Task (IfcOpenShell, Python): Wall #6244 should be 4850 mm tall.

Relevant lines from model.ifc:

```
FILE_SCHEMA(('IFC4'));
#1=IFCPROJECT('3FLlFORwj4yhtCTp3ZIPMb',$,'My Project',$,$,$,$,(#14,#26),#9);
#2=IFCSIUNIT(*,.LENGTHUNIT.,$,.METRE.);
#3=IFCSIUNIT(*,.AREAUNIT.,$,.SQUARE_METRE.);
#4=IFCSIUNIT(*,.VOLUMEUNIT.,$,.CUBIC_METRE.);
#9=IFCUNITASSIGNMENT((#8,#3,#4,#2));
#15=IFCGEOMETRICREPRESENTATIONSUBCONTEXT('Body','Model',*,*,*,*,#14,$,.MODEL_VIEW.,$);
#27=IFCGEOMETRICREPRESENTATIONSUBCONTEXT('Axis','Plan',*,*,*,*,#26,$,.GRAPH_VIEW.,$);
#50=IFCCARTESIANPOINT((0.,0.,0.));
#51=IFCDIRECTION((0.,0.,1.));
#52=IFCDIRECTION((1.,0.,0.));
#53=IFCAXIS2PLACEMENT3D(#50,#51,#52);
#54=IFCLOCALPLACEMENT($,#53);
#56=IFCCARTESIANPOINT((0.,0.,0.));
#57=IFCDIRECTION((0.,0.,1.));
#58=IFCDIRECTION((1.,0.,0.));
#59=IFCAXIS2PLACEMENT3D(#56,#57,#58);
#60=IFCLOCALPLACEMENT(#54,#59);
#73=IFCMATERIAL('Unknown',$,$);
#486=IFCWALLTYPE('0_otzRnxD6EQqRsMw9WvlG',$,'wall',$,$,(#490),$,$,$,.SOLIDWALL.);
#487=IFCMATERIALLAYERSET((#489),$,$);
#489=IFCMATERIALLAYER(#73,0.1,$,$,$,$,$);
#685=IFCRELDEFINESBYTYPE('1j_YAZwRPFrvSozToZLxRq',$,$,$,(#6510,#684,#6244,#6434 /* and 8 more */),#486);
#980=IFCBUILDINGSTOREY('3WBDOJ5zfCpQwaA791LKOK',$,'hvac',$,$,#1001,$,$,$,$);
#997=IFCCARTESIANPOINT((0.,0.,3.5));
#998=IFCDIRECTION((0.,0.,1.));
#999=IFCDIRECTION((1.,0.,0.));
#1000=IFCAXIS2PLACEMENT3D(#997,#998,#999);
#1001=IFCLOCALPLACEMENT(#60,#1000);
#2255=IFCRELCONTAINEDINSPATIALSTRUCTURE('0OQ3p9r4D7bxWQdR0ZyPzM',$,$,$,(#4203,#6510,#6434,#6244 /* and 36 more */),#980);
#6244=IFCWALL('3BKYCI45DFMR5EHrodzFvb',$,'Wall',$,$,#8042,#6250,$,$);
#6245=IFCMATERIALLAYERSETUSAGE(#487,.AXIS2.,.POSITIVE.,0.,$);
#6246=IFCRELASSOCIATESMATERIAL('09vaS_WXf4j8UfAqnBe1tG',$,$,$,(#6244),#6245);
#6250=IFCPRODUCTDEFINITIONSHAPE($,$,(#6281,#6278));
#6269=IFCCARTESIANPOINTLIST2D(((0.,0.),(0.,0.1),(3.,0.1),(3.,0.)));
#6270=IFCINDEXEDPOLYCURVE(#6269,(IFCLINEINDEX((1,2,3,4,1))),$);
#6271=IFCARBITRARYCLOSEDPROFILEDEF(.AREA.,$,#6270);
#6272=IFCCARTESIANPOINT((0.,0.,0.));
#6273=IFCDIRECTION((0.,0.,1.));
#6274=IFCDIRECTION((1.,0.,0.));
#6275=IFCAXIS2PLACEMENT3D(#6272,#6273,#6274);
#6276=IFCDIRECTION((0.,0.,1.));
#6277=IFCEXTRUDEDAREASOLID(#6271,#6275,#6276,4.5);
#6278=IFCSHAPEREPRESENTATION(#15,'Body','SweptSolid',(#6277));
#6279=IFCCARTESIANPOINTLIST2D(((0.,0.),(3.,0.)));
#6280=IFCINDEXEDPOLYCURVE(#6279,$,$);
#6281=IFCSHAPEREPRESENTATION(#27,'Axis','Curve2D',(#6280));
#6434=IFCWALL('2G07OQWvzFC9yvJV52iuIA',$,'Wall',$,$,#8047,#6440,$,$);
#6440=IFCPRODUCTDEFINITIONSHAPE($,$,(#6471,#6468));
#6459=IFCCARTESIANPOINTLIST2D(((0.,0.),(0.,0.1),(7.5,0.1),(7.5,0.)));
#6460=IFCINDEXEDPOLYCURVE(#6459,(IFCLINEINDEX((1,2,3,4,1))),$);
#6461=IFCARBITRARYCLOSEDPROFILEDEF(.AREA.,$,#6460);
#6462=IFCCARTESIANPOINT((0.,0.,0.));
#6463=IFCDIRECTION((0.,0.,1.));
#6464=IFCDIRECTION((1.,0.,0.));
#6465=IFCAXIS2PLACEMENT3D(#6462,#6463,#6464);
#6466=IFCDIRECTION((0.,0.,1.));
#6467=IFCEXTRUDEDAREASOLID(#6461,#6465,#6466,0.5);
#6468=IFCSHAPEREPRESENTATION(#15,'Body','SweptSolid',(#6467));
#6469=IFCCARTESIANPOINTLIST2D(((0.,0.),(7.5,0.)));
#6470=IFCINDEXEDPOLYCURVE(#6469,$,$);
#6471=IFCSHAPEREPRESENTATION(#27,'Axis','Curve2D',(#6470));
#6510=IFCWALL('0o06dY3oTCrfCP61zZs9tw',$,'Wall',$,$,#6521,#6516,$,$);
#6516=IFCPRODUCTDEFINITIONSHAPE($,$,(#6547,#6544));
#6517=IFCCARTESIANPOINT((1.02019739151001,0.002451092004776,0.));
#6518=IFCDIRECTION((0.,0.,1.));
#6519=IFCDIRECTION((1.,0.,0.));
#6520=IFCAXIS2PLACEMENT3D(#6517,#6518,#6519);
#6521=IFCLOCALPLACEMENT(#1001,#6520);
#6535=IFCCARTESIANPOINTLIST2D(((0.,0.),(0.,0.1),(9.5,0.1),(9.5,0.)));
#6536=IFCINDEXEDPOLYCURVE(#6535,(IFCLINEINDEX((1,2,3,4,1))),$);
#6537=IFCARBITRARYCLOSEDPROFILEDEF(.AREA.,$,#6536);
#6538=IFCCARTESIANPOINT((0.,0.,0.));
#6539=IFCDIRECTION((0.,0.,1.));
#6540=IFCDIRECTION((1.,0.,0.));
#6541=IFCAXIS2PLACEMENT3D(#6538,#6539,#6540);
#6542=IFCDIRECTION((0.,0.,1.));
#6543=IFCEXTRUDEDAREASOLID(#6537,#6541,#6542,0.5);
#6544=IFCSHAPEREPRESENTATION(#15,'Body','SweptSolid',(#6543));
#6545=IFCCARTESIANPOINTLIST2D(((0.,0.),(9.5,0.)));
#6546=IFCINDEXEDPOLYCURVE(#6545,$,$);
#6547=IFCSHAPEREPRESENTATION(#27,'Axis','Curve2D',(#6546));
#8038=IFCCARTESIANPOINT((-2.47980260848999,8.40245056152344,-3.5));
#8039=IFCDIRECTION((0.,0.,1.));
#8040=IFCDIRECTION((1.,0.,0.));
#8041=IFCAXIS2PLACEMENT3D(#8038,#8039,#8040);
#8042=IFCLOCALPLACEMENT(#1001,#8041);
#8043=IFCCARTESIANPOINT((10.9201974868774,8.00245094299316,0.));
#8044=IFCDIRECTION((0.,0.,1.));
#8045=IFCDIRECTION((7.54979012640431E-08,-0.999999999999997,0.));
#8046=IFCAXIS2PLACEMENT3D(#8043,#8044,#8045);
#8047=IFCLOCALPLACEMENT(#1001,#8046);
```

```python
import ifcopenshell
import ifcopenshell.geom
import ifcopenshell.util.representation
import ifcopenshell.util.shape
import ifcopenshell.util.unit

model = ifcopenshell.open("model.ifc")
unit_scale = ifcopenshell.util.unit.calculate_unit_scale(model)
settings = ifcopenshell.geom.settings()


def volume(element):
    """Net volume in cubic metres, openings subtracted."""
    shape = ifcopenshell.geom.create_shape(settings, element)
    return ifcopenshell.util.shape.get_volume(shape.geometry)


wall = model.by_id(6244)
before = volume(wall)

body = ifcopenshell.util.representation.get_representation(wall, "Model", "Body")
solid = body.Items[0]
old_height = solid.Depth
solid.Depth = 4.85 / unit_scale
after = volume(wall)

print(f"height {old_height:g} -> {solid.Depth:g}, volume {before:.3f} -> {after:.3f} m3")

model.write("model_rev.ifc")
```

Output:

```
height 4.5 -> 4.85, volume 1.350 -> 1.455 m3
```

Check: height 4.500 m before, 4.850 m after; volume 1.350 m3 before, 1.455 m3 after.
